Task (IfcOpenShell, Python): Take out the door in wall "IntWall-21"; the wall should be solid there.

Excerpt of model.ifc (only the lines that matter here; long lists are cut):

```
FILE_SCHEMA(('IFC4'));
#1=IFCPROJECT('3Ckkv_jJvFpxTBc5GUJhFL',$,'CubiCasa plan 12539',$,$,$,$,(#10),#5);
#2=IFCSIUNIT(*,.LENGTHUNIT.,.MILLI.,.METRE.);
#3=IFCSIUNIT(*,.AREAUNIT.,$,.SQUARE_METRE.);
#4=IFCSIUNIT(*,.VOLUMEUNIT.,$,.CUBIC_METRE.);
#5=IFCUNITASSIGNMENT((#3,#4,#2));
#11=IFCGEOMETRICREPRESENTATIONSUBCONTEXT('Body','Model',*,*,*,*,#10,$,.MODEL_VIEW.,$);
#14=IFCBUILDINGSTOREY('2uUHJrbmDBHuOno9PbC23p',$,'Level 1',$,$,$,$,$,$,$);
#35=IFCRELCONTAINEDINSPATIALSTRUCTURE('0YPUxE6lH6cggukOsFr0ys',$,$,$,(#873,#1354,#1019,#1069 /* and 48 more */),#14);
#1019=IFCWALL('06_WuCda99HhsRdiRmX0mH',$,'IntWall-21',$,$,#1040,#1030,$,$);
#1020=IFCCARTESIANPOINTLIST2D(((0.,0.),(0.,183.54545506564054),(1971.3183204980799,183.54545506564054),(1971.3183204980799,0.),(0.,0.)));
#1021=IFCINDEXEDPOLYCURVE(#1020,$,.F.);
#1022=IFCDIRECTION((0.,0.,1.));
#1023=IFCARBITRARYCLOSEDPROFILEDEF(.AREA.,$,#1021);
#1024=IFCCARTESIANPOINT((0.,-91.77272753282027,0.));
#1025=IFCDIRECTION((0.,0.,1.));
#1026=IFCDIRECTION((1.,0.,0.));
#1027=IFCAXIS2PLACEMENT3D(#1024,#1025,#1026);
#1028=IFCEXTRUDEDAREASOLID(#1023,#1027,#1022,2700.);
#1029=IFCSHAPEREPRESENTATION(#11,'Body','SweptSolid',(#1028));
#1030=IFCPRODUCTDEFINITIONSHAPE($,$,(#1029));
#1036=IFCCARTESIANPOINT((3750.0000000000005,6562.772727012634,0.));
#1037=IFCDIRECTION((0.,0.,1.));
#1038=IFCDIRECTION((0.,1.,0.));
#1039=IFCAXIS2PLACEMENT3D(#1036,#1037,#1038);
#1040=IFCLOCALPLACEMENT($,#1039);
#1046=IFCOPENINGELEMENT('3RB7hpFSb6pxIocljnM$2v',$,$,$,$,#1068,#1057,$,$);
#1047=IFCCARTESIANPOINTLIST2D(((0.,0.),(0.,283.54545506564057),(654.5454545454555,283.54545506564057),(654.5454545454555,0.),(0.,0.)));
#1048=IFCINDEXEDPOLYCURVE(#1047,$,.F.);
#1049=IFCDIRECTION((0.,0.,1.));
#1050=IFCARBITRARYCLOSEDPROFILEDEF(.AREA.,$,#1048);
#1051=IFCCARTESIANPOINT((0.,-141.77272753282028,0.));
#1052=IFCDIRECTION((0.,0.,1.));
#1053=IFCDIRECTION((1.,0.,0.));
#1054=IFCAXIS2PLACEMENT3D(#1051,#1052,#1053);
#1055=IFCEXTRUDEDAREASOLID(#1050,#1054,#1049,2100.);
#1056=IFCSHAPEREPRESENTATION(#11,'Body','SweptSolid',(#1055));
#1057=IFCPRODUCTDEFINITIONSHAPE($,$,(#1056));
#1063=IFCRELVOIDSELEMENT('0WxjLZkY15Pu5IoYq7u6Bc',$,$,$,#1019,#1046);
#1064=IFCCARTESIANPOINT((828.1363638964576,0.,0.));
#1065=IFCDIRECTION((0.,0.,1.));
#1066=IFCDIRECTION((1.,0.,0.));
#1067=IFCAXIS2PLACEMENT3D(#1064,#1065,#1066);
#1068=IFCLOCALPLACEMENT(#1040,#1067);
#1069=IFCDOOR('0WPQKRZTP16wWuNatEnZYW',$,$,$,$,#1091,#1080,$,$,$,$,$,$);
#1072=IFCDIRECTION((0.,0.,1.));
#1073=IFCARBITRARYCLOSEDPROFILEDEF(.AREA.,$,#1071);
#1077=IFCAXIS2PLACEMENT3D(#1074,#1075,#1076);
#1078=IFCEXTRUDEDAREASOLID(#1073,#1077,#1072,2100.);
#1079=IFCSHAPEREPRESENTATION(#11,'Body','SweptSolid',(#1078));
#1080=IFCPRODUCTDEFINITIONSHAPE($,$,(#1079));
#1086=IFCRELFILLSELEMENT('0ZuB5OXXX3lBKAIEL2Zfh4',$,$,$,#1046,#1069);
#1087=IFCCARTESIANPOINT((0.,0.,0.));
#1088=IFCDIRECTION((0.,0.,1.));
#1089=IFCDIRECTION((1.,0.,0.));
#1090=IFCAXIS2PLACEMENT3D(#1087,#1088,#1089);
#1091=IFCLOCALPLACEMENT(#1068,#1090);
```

```python
import ifcopenshell
import ifcopenshell.api.feature
import ifcopenshell.api.root
import ifcopenshell.geom
import ifcopenshell.util.shape

model = ifcopenshell.open("model.ifc")
settings = ifcopenshell.geom.settings()


def volume(element):
    """Net volume in cubic metres, openings subtracted."""
    shape = ifcopenshell.geom.create_shape(settings, element)
    return ifcopenshell.util.shape.get_volume(shape.geometry)


door = model.by_guid("0WPQKRZTP16wWuNatEnZYW")
opening = door.FillsVoids[0].RelatingOpeningElement
wall = opening.VoidsElements[0].RelatingBuildingElement
before = volume(wall)

ifcopenshell.api.root.remove_product(model, product=door)
ifcopenshell.api.feature.remove_feature(model, feature=opening)

after = volume(wall)

print(f"wall volume {before:.3f} -> {after:.3f} m3")

model.write("model-out.ifc")
```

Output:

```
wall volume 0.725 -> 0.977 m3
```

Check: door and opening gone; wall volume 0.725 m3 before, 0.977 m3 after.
